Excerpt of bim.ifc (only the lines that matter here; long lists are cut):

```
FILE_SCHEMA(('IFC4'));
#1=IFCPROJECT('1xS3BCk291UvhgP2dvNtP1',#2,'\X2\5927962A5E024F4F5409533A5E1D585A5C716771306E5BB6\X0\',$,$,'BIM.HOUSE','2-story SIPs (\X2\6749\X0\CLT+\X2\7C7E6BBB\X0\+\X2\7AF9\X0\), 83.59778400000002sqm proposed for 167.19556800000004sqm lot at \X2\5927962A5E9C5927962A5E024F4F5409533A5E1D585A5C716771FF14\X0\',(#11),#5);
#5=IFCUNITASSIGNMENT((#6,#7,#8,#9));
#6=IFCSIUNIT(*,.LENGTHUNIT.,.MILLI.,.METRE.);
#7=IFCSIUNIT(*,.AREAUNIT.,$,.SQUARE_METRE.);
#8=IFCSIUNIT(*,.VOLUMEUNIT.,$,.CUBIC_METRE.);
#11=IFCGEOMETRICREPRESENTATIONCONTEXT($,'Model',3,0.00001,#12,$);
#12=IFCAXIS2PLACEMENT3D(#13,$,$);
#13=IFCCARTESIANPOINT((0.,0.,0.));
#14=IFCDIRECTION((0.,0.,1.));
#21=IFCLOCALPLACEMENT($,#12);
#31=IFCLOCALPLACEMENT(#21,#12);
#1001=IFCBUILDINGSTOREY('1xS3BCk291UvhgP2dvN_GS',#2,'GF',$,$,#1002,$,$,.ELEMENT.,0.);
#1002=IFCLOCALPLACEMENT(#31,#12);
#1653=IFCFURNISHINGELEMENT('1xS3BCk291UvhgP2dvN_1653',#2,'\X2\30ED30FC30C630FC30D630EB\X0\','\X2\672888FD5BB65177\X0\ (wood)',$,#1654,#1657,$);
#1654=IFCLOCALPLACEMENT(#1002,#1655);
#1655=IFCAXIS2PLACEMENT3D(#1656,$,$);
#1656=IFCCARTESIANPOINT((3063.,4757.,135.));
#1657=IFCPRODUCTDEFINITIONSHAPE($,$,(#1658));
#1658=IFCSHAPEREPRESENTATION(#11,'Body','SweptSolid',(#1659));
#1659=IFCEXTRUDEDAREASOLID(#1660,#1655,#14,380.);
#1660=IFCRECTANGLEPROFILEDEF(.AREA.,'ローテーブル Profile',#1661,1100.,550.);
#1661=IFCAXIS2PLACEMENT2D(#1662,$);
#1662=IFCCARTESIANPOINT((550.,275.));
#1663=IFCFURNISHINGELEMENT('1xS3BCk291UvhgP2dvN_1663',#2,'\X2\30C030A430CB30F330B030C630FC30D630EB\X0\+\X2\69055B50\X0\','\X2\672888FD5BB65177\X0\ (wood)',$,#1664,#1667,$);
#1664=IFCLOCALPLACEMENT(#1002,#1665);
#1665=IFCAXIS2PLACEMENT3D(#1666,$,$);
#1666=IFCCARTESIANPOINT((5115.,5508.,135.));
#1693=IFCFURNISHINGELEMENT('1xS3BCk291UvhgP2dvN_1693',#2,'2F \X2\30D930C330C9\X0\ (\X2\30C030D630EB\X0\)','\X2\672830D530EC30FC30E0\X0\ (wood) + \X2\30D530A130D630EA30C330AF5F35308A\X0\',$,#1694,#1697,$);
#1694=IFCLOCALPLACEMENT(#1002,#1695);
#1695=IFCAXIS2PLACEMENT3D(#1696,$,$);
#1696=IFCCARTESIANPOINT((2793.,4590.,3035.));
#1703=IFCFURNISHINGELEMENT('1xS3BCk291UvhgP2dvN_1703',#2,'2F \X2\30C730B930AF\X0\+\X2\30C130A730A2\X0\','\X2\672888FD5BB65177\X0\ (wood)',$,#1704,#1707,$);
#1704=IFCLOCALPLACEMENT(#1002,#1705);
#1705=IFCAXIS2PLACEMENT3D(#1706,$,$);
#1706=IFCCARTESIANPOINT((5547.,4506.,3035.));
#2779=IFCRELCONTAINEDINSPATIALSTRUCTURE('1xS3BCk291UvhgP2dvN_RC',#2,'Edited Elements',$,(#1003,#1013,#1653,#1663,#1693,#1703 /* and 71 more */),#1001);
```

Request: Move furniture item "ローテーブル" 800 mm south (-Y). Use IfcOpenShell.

```python
import ifcopenshell
import ifcopenshell.api.geometry
import ifcopenshell.util.placement
import ifcopenshell.util.unit

model = ifcopenshell.open("bim.ifc")
unit_scale = ifcopenshell.util.unit.calculate_unit_scale(model)

item = model.by_guid("1xS3BCk291UvhgP2dvN_1653")
matrix = ifcopenshell.util.placement.get_local_placement(item.ObjectPlacement)
matrix[1, 3] -= 0.8 / unit_scale
ifcopenshell.api.geometry.edit_object_placement(model, product=item, matrix=matrix, is_si=False)

print(ifcopenshell.util.placement.get_local_placement(item.ObjectPlacement).round(3) + 0.0)

model.write("bim-out.ifc")
```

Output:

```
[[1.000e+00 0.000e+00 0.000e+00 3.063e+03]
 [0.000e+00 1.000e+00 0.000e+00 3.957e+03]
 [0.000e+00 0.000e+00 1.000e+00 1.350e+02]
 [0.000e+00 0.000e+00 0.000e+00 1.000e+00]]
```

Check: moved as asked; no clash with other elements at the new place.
